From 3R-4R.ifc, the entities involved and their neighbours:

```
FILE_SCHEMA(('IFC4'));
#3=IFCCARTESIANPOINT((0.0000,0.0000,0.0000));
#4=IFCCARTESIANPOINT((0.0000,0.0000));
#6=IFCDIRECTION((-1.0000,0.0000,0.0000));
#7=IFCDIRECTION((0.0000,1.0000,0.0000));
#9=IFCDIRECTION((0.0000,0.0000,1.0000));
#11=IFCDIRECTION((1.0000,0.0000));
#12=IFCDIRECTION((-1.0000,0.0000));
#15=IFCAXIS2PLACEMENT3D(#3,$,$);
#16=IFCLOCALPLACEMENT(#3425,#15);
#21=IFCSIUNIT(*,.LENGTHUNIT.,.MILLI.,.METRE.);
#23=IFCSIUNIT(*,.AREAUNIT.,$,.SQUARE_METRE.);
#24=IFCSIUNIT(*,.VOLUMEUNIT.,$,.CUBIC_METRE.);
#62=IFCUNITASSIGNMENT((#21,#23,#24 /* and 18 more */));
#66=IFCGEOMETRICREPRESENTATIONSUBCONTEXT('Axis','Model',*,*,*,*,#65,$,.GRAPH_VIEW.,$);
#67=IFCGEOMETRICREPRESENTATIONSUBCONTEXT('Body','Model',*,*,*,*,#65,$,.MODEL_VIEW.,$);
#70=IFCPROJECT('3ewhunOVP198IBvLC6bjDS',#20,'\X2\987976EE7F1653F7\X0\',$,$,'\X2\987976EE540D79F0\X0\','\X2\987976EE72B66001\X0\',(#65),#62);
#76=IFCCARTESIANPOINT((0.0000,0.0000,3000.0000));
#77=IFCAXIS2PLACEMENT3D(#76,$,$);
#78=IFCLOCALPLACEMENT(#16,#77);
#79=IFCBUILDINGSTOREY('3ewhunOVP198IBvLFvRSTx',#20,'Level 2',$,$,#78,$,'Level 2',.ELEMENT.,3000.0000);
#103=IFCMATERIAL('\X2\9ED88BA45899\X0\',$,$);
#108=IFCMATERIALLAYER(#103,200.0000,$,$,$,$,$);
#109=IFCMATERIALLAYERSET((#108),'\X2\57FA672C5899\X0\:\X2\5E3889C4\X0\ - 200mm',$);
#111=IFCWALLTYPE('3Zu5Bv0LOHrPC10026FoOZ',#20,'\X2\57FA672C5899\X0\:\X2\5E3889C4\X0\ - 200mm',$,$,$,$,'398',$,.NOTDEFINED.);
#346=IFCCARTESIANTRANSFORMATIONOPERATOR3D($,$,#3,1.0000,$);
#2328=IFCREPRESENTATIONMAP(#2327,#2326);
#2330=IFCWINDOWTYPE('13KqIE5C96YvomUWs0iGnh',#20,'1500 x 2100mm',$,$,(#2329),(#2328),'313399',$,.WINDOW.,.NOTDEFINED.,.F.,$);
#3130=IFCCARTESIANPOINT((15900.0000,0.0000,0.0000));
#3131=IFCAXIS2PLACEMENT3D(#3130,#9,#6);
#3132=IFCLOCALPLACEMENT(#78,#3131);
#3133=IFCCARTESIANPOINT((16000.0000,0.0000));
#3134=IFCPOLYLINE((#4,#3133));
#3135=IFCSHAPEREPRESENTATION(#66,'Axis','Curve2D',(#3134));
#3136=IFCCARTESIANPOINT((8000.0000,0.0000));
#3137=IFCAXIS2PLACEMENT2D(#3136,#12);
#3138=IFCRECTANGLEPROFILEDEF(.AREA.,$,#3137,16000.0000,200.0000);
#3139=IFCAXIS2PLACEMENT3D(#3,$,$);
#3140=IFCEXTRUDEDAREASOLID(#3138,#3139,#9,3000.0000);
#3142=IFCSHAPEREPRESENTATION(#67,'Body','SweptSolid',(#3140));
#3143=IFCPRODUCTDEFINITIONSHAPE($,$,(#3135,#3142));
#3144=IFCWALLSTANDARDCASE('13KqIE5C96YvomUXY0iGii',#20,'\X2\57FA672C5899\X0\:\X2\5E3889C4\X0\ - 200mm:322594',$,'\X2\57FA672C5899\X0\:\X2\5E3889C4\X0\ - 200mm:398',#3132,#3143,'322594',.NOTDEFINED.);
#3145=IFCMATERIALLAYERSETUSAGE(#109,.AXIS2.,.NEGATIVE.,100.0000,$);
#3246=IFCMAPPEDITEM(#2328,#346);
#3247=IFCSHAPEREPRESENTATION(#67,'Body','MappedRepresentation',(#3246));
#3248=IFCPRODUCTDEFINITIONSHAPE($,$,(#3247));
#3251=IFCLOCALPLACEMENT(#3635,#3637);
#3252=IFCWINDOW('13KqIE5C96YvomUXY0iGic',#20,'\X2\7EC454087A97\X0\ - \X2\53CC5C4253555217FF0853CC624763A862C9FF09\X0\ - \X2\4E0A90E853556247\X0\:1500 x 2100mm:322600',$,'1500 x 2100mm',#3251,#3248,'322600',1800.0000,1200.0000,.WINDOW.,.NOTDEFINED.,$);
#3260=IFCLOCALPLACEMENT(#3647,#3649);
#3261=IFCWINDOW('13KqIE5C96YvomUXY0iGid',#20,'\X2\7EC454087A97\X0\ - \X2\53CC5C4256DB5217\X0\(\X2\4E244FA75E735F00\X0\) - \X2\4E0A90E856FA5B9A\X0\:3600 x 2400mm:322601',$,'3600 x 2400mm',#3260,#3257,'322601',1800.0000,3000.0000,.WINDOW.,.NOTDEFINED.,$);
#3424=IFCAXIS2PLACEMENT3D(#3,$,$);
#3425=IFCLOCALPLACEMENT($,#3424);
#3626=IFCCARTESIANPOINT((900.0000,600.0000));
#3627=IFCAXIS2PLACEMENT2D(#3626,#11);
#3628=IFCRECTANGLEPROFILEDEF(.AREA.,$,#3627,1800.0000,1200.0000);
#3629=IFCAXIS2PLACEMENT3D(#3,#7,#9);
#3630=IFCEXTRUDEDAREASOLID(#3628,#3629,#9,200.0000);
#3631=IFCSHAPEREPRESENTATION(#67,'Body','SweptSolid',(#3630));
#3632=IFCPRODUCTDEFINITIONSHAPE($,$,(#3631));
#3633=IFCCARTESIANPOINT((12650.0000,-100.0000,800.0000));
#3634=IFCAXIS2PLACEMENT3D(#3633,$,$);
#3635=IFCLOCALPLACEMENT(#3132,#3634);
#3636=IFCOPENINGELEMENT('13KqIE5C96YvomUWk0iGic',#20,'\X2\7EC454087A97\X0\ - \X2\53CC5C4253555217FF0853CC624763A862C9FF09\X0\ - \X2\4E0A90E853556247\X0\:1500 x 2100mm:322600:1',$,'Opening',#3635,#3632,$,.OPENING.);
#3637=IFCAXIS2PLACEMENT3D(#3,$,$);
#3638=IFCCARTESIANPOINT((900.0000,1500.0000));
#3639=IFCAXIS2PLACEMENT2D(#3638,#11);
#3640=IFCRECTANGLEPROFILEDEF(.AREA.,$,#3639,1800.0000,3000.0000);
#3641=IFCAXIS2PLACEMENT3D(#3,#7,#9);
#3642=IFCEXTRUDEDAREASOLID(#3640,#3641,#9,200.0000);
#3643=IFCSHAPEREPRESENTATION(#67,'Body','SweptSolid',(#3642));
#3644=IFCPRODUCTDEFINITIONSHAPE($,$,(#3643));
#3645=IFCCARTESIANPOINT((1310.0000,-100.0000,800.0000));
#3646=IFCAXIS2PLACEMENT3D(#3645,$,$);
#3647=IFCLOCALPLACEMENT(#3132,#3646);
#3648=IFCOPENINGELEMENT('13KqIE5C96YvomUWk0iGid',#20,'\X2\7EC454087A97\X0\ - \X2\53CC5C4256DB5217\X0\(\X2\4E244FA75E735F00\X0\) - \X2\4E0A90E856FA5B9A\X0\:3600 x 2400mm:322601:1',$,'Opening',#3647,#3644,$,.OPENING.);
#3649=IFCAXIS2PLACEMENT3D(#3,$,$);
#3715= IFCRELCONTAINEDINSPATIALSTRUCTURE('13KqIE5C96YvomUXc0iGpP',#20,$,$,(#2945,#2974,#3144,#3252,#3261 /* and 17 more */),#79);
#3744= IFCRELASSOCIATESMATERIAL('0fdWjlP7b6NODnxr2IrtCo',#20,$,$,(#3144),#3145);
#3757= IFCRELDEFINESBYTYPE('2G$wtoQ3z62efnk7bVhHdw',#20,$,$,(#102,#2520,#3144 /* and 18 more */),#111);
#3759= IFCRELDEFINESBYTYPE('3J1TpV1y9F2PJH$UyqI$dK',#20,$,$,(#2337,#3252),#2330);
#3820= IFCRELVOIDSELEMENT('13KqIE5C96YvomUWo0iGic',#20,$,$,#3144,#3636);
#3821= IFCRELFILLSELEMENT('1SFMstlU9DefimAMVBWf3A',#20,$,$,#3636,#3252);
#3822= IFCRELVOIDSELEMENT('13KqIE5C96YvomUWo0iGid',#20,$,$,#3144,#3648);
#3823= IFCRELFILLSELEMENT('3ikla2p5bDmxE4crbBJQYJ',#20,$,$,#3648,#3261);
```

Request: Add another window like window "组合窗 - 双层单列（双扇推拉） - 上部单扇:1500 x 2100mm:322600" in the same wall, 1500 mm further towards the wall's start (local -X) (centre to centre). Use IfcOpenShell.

```python
import ifcopenshell
import ifcopenshell.api.feature
import ifcopenshell.api.geometry
import ifcopenshell.api.root
import ifcopenshell.geom
import ifcopenshell.util.element
import ifcopenshell.util.placement
import ifcopenshell.util.shape

model = ifcopenshell.open("3R-4R.ifc")
settings = ifcopenshell.geom.settings()


def volume(element):
    """Net volume in cubic metres, openings subtracted."""
    shape = ifcopenshell.geom.create_shape(settings, element)
    return ifcopenshell.util.shape.get_volume(shape.geometry)


def reuse_history(source, copy):
    """copy_class also copies each property set's owner history, people and application; keep the originals."""
    for rel in copy.IsDefinedBy:
        if rel.is_a("IfcRelDefinesByProperties") and (history := rel.RelatingPropertyDefinition.OwnerHistory):
            rel.RelatingPropertyDefinition.OwnerHistory = source.OwnerHistory
            ifcopenshell.util.element.remove_deep2(model, history)


window = model.by_id(3252)
opening = window.FillsVoids[0].RelatingOpeningElement
wall = opening.VoidsElements[0].RelatingBuildingElement
before = volume(wall)
shift = ifcopenshell.util.placement.get_local_placement(wall.ObjectPlacement)[:3, 0] * -1500.0

# copy_class copies the void relationship, type, container and properties, but no geometry.
new_opening = ifcopenshell.api.root.copy_class(model, product=opening)
new_opening.Representation = ifcopenshell.util.element.copy_deep(
    model, opening.Representation, exclude=["IfcGeometricRepresentationContext", "IfcRepresentationMap"]
)
new_opening.Name = "组合窗 - 双层单列（双扇推拉） - 上部单扇:1500 x 2100mm"
new_window = ifcopenshell.api.root.copy_class(model, product=window)
new_window.Representation = ifcopenshell.util.element.copy_deep(
    model, window.Representation, exclude=["IfcGeometricRepresentationContext", "IfcRepresentationMap"]
)
new_window.Name = "组合窗 - 双层单列（双扇推拉） - 上部单扇:1500 x 2100mm"
new_window.Tag = None
reuse_history(window, new_window)
ifcopenshell.api.feature.add_filling(model, opening=new_opening, element=new_window)

for old, new in ((opening, new_opening), (window, new_window)):
    matrix = ifcopenshell.util.placement.get_local_placement(old.ObjectPlacement)
    matrix[:3, 3] += shift
    ifcopenshell.api.geometry.edit_object_placement(model, product=new, matrix=matrix, is_si=False)

after = volume(wall)

print(f"wall volume {before:.3f} -> {after:.3f} m3")

model.write("3R-4R_edited.ifc")
```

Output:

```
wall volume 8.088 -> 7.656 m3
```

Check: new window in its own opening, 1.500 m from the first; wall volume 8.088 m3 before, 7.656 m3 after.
